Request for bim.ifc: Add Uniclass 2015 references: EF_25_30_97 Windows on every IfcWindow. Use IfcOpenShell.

First a look at what the model holds.

```python
import ifcopenshell

model = ifcopenshell.open("bim.ifc")
print(model.schema)
print("classifications:", [c.Name for c in model.by_type("IfcClassification")])
for ifc_class in ("IfcDoor", "IfcRoof", "IfcStair", "IfcWall", "IfcWindow"):
    print(ifc_class, len(model.by_type(ifc_class)))
```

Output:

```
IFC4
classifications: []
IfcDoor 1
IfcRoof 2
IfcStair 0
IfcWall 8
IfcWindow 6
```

```python
import ifcopenshell
import ifcopenshell.api.classification

model = ifcopenshell.open("bim.ifc")

system = ifcopenshell.api.classification.add_classification(model, classification="Uniclass 2015")

codes = {
    "IfcWindow": ("EF_25_30_97", "Windows"),
}
for ifc_class, (code, name) in codes.items():
    products = model.by_type(ifc_class)
    ifcopenshell.api.classification.add_reference(
        model, products=products, classification=system, identification=code, name=name
    )
    print(code, len(products))

model.write("bim_edited.ifc")
```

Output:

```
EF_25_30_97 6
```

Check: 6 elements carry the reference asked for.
